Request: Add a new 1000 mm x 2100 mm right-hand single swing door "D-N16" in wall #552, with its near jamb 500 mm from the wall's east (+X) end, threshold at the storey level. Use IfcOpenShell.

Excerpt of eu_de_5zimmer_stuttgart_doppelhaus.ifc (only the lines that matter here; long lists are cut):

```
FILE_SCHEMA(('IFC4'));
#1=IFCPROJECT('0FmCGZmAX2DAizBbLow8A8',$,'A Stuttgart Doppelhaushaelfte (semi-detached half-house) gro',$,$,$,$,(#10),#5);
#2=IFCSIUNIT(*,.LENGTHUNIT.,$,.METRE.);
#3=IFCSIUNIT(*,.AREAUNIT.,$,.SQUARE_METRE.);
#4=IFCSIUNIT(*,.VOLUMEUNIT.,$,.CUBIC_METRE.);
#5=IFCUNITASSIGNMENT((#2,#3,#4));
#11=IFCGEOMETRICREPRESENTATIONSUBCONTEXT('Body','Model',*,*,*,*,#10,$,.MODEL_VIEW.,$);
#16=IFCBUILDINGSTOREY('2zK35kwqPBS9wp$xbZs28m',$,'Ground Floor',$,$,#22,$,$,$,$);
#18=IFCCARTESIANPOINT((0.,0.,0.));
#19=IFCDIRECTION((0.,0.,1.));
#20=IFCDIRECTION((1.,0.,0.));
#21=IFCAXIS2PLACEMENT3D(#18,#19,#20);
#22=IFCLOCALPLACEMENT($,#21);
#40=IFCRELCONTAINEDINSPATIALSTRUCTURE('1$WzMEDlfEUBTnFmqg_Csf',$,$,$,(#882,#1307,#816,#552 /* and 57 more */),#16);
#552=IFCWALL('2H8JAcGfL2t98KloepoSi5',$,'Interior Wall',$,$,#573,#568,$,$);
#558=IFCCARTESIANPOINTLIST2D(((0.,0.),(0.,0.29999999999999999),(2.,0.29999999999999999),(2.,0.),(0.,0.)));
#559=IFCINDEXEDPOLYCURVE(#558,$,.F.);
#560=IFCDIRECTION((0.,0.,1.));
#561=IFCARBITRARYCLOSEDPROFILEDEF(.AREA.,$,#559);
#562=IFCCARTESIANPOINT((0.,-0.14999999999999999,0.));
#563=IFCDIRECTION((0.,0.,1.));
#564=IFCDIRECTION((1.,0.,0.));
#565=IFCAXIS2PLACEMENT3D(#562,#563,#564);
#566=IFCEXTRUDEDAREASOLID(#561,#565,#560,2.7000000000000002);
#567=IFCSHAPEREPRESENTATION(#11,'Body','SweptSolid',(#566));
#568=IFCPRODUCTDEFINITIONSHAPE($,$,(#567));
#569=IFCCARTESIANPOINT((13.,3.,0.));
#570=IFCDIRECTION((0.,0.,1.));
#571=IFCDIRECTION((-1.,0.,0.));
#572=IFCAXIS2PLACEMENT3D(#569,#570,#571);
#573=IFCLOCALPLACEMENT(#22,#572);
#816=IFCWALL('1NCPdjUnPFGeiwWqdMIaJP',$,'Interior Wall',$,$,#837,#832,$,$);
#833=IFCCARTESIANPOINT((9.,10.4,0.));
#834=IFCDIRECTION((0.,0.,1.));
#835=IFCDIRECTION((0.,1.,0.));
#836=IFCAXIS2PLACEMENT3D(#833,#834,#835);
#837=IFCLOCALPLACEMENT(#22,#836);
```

```python
import numpy as np
import ifcopenshell
import ifcopenshell.api.feature
import ifcopenshell.api.geometry
import ifcopenshell.api.root
import ifcopenshell.api.spatial
import ifcopenshell.geom
import ifcopenshell.util.element
import ifcopenshell.util.placement
import ifcopenshell.util.representation
import ifcopenshell.util.shape
import ifcopenshell.util.unit

model = ifcopenshell.open("eu_de_5zimmer_stuttgart_doppelhaus.ifc")
unit_scale = ifcopenshell.util.unit.calculate_unit_scale(model)
settings = ifcopenshell.geom.settings()


def volume(element):
    """Net volume in cubic metres, openings subtracted."""
    shape = ifcopenshell.geom.create_shape(settings, element)
    return ifcopenshell.util.shape.get_volume(shape.geometry)


wall = model.by_id(552)
storey = ifcopenshell.util.element.get_container(wall, ifc_class="IfcBuildingStorey")
context = ifcopenshell.util.representation.get_context(model, "Model", "Body", "MODEL_VIEW")
before = volume(wall)

width, height, from_end, sill = 1, 2.1, 0.5, 0.0  # metres

# The wall runs along its own X axis, and the end named is its -X end.
wall_shape = ifcopenshell.geom.create_shape(settings, wall)
x, y, z = ifcopenshell.util.shape.get_vertices(wall_shape.geometry).T
start = x.min() + from_end
face, thickness = float(y.min()), float(y.max() - y.min())
wall_matrix = ifcopenshell.util.placement.get_local_placement(wall.ObjectPlacement)
level = ifcopenshell.util.placement.get_local_placement(storey.ObjectPlacement)[2, 3]


def in_wall(x, y):
    """Placement at x, y metres in the wall's axes, at sill height."""
    matrix = wall_matrix.copy()
    matrix[:, 3] = wall_matrix @ np.array([x / unit_scale, y / unit_scale, 0.0, 1.0])
    matrix[2, 3] = level + sill / unit_scale
    return matrix


# Opening: a box that overshoots both wall faces by 50 mm.
opening = ifcopenshell.api.root.create_entity(model, ifc_class="IfcOpeningElement", predefined_type="OPENING")
box = ifcopenshell.api.geometry.add_wall_representation(
    model, context=context, length=width, height=height, thickness=thickness + 0.1
)
ifcopenshell.api.geometry.assign_representation(model, product=opening, representation=box)
ifcopenshell.api.geometry.edit_object_placement(model, product=opening, matrix=in_wall(start, face - 0.05), is_si=False)
ifcopenshell.api.feature.add_feature(model, feature=opening, element=wall)

door = ifcopenshell.api.root.create_entity(model, ifc_class="IfcDoor", name="D-N16", predefined_type="DOOR")
door.OverallWidth, door.OverallHeight = width / unit_scale, height / unit_scale
door.OperationType = "SINGLE_SWING_RIGHT"
body = ifcopenshell.api.geometry.add_door_representation(
    model,
    context=context,
    overall_width=door.OverallWidth,
    overall_height=door.OverallHeight,
    operation_type="SINGLE_SWING_RIGHT",
    lining_properties={"LiningDepth": thickness / unit_scale, "ThresholdDepth": thickness / unit_scale},
)
ifcopenshell.api.geometry.assign_representation(model, product=door, representation=body)
ifcopenshell.api.spatial.assign_container(model, products=[door], relating_structure=storey)
ifcopenshell.api.feature.add_filling(model, opening=opening, element=door)

# The lining spans the wall, so the door starts at the wall face.
ifcopenshell.api.geometry.edit_object_placement(model, product=door, matrix=in_wall(start, face), is_si=False)

after = volume(wall)

print(f"wall volume {before:.3f} -> {after:.3f} m3")

model.write("eu_de_5zimmer_stuttgart_doppelhaus_updated.ifc")
```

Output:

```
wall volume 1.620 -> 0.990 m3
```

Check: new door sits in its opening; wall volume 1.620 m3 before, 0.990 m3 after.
